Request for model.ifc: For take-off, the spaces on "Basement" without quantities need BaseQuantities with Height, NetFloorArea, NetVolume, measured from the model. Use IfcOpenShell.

First a look at what the model holds.

```python
import ifcopenshell
import ifcopenshell.util.element
import ifcopenshell.util.unit

model = ifcopenshell.open("model.ifc")
print(model.schema)
for unit_type in ("LENGTHUNIT", "AREAUNIT", "VOLUMEUNIT"):
    print(unit_type, ifcopenshell.util.unit.calculate_unit_scale(model, unit_type))
storey = next(s for s in model.by_type("IfcBuildingStorey") if s.Name == "Basement")
spaces = [e for e in ifcopenshell.util.element.get_decomposition(storey) if e.is_a("IfcSpace")]
for e in sorted(spaces, key=lambda e: e.id()):
    print(e.id(), e.is_a(), e.Name, list(ifcopenshell.util.element.get_psets(e, qtos_only=True)), sep=" | ")
```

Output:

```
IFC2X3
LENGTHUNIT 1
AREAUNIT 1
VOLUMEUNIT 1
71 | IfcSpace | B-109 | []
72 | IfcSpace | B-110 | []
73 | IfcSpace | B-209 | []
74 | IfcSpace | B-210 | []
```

```python
import ifcopenshell
import ifcopenshell.api.pset
import ifcopenshell.geom
import ifcopenshell.util.element
import ifcopenshell.util.shape
import ifcopenshell.util.unit

model = ifcopenshell.open("model.ifc")
unit_scale = ifcopenshell.util.unit.calculate_unit_scale(model)
area_scale = ifcopenshell.util.unit.calculate_unit_scale(model, "AREAUNIT")
volume_scale = ifcopenshell.util.unit.calculate_unit_scale(model, "VOLUMEUNIT")
settings = ifcopenshell.geom.settings()

storey = next(s for s in model.by_type("IfcBuildingStorey") if s.Name == "Basement")
spaces = [e for e in ifcopenshell.util.element.get_decomposition(storey) if e.is_a("IfcSpace")]

for e in sorted(spaces, key=lambda e: e.id()):
    if ifcopenshell.util.element.get_psets(e, qtos_only=True, should_inherit=False):
        continue
    # Geometry comes back in metres, in the element's own axes.
    shape = ifcopenshell.geom.create_shape(settings, e)
    values = {
        "Height": ifcopenshell.util.shape.get_z(shape.geometry) / unit_scale,
        "NetFloorArea": ifcopenshell.util.shape.get_footprint_area(shape.geometry) / area_scale,
        "NetVolume": ifcopenshell.util.shape.get_volume(shape.geometry) / volume_scale,
    }
    qto = ifcopenshell.api.pset.add_qto(model, product=e, name="BaseQuantities")
    ifcopenshell.api.pset.edit_qto(model, qto=qto, properties=values)
    print(e.id(), {k: round(v, 3) for k, v in values.items()})

model.write("model-out.ifc")
```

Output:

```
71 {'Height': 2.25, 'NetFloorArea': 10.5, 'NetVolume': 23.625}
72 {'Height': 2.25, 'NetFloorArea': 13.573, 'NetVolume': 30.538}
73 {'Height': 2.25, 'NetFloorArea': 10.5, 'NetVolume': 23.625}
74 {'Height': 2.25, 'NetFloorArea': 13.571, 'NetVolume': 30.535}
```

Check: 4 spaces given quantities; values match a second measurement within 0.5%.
